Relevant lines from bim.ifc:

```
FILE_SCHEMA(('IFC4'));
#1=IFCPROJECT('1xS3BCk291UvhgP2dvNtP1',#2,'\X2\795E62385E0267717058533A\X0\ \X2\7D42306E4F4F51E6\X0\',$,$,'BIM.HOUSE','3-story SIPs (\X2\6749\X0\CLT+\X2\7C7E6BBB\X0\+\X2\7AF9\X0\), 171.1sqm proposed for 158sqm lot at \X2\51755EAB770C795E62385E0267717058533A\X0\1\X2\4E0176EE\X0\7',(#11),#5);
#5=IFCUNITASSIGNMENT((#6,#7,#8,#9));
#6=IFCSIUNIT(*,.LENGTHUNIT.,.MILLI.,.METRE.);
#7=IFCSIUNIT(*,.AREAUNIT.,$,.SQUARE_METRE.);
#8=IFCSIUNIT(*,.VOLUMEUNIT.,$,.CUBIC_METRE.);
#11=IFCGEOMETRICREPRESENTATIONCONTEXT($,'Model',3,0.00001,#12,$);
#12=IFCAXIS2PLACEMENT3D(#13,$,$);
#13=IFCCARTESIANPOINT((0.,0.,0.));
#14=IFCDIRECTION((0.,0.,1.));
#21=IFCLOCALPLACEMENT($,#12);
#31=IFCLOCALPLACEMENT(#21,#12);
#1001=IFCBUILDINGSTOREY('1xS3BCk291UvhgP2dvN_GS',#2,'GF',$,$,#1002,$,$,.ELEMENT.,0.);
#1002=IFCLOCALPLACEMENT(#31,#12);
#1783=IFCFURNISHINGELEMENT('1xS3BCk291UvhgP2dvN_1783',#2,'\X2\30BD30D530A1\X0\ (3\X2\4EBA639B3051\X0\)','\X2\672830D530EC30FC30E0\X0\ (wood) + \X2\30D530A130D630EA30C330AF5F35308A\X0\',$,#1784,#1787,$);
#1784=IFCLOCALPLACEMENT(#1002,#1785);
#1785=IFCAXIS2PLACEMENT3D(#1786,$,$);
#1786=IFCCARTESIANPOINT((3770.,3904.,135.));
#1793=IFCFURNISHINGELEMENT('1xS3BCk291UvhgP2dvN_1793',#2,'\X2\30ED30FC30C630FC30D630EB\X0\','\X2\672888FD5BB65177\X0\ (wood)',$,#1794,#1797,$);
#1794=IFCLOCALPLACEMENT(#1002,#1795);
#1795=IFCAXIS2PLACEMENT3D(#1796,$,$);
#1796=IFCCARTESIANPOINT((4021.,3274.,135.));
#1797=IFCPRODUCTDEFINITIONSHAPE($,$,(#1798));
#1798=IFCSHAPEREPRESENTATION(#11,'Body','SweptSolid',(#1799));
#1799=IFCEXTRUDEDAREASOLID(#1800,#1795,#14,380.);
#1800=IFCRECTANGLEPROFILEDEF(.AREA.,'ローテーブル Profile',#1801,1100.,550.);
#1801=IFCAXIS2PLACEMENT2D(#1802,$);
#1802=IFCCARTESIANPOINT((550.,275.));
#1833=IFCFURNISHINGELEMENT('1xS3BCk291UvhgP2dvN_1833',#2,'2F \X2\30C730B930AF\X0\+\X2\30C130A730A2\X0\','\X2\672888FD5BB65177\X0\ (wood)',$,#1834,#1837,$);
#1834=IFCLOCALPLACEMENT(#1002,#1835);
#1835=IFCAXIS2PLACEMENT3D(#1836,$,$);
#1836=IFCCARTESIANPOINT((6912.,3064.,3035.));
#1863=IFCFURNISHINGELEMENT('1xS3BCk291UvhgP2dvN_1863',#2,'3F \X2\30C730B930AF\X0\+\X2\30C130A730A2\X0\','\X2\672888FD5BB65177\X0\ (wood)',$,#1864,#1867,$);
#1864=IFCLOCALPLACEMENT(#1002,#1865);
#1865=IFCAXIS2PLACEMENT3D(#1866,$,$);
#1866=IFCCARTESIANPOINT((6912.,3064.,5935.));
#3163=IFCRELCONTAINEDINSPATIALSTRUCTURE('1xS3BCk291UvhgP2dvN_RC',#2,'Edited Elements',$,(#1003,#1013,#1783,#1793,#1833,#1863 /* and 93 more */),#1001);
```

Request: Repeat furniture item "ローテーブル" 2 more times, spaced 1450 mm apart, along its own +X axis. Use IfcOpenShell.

```python
import ifcopenshell
import ifcopenshell.api.geometry
import ifcopenshell.api.root
import ifcopenshell.util.element
import ifcopenshell.util.placement

model = ifcopenshell.open("bim.ifc")


def reuse_history(source, copy):
    """copy_class also copies each property set's owner history, people and application; keep the originals."""
    for rel in copy.IsDefinedBy:
        if rel.is_a("IfcRelDefinesByProperties") and (history := rel.RelatingPropertyDefinition.OwnerHistory):
            rel.RelatingPropertyDefinition.OwnerHistory = source.OwnerHistory
            ifcopenshell.util.element.remove_deep2(model, history)


source = model.by_guid("1xS3BCk291UvhgP2dvN_1793")
base = ifcopenshell.util.placement.get_local_placement(source.ObjectPlacement)
step = base[:3, 0] * 1450.0

for i in range(1, 3):
    copy = ifcopenshell.api.root.copy_class(model, product=source)
    copy.Representation = ifcopenshell.util.element.copy_deep(
        model, source.Representation, exclude=["IfcGeometricRepresentationContext", "IfcRepresentationMap"]
    )
    reuse_history(source, copy)
    matrix = base.copy()
    matrix[:3, 3] += i * step
    print("added at", matrix[:3, 3].round(3) + 0.0)
    ifcopenshell.api.geometry.edit_object_placement(model, product=copy, matrix=matrix, is_si=False)

model.write("bim_rev.ifc")
```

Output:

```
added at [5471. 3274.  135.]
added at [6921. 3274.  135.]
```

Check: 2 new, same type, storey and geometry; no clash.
